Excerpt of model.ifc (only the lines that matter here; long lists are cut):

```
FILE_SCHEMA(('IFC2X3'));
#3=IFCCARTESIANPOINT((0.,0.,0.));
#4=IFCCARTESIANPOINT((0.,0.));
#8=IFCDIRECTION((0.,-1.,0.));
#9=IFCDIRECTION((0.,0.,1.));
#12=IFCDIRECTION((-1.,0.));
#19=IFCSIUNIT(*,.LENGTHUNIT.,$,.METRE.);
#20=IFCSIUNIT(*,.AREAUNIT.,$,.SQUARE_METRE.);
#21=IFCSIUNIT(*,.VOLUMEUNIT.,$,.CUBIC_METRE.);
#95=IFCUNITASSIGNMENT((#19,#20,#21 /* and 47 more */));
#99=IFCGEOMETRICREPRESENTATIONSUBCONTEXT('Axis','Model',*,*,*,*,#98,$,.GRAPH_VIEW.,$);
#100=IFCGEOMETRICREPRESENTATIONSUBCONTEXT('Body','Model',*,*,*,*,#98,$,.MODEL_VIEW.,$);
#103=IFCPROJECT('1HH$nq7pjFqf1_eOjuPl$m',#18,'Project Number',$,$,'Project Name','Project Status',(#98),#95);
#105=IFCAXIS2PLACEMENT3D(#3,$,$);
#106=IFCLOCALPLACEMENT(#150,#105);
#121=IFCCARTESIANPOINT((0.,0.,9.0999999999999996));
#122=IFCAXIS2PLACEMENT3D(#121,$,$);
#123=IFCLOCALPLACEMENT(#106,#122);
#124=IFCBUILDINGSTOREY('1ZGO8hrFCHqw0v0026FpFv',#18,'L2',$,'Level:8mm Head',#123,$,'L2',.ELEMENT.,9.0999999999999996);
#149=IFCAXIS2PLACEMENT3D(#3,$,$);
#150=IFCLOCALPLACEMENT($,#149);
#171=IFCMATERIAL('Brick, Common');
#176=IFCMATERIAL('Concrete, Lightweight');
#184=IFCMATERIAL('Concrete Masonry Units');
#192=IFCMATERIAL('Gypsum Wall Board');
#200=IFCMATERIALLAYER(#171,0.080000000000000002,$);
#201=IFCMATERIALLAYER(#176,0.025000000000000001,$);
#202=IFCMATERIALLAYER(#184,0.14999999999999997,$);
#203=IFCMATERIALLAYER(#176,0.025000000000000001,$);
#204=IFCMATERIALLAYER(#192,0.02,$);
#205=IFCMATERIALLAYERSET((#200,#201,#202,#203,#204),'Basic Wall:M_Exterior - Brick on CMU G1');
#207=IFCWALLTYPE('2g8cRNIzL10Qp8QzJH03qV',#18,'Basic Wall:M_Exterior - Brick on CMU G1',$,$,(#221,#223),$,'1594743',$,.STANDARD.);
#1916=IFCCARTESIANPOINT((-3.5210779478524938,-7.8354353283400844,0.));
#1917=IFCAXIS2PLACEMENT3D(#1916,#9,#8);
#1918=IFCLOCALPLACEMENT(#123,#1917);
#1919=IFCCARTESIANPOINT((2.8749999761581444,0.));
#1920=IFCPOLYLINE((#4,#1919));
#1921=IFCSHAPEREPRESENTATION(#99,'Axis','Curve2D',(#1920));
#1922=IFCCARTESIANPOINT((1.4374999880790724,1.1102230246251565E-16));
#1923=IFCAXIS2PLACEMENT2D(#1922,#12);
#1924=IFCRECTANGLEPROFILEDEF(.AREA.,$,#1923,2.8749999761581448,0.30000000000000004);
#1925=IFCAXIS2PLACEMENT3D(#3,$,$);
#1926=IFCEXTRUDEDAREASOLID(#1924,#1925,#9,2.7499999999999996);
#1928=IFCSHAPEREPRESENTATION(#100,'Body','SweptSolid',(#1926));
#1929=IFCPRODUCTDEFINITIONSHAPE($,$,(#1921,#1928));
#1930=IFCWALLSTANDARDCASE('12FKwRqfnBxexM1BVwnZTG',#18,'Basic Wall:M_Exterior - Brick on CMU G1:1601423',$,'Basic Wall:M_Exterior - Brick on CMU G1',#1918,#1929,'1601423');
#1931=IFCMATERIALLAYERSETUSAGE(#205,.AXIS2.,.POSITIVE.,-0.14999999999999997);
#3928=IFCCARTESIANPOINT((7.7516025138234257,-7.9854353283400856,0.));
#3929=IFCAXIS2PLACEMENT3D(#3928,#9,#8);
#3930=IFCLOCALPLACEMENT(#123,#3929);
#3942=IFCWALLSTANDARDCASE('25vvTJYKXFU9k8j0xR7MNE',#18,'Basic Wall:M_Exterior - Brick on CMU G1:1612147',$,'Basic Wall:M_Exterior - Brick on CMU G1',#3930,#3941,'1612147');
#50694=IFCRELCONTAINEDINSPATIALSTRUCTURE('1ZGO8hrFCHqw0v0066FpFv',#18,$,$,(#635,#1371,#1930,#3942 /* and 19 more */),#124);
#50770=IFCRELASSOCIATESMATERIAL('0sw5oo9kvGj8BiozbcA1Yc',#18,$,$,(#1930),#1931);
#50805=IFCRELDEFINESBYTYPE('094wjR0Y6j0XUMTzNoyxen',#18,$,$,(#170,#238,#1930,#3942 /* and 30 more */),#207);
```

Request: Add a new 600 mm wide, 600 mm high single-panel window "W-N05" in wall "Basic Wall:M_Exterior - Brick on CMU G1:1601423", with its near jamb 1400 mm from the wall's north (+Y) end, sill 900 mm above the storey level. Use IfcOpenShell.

```python
import numpy as np
import ifcopenshell
import ifcopenshell.api.feature
import ifcopenshell.api.geometry
import ifcopenshell.api.root
import ifcopenshell.api.spatial
import ifcopenshell.api.type
import ifcopenshell.geom
import ifcopenshell.util.element
import ifcopenshell.util.placement
import ifcopenshell.util.representation
import ifcopenshell.util.shape
import ifcopenshell.util.unit

model = ifcopenshell.open("model.ifc")
unit_scale = ifcopenshell.util.unit.calculate_unit_scale(model)
settings = ifcopenshell.geom.settings()


def volume(element):
    """Net volume in cubic metres, openings subtracted."""
    shape = ifcopenshell.geom.create_shape(settings, element)
    return ifcopenshell.util.shape.get_volume(shape.geometry)


wall = model.by_guid("12FKwRqfnBxexM1BVwnZTG")
storey = ifcopenshell.util.element.get_container(wall, ifc_class="IfcBuildingStorey")
context = ifcopenshell.util.representation.get_context(model, "Model", "Body", "MODEL_VIEW")
before = volume(wall)

width, height, from_end, sill = 0.6, 0.6, 1.4, 0.9  # metres

# The wall runs along its own X axis, and the end named is its -X end.
wall_shape = ifcopenshell.geom.create_shape(settings, wall)
x, y, z = ifcopenshell.util.shape.get_vertices(wall_shape.geometry).T
start = x.min() + from_end
face, thickness = float(y.min()), float(y.max() - y.min())
wall_matrix = ifcopenshell.util.placement.get_local_placement(wall.ObjectPlacement)
level = ifcopenshell.util.placement.get_local_placement(storey.ObjectPlacement)[2, 3]


def in_wall(x, y):
    """Placement at x, y metres in the wall's axes, at sill height."""
    matrix = wall_matrix.copy()
    matrix[:, 3] = wall_matrix @ np.array([x / unit_scale, y / unit_scale, 0.0, 1.0])
    matrix[2, 3] = level + sill / unit_scale
    return matrix


# Opening: a box that overshoots both wall faces by 50 mm.
opening = ifcopenshell.api.root.create_entity(model, ifc_class="IfcOpeningElement")
box = ifcopenshell.api.geometry.add_wall_representation(
    model, context=context, length=width, height=height, thickness=thickness + 0.1
)
ifcopenshell.api.geometry.assign_representation(model, product=opening, representation=box)
ifcopenshell.api.geometry.edit_object_placement(model, product=opening, matrix=in_wall(start, face - 0.05), is_si=False)
ifcopenshell.api.feature.add_feature(model, feature=opening, element=wall)

window = ifcopenshell.api.root.create_entity(model, ifc_class="IfcWindow", name="W-N05")
window.OverallWidth, window.OverallHeight = width / unit_scale, height / unit_scale
body = ifcopenshell.api.geometry.add_window_representation(
    model,
    context=context,
    overall_width=window.OverallWidth,
    overall_height=window.OverallHeight,
    partition_type="SINGLE_PANEL",
)
ifcopenshell.api.geometry.assign_representation(model, product=window, representation=body)
ifcopenshell.api.spatial.assign_container(model, products=[window], relating_structure=storey)
fills = ifcopenshell.api.feature.add_filling(model, opening=opening, element=window)
fills.OwnerHistory = window.OwnerHistory  # required in IFC2X3

# IFC2X3 keeps the operation on the window style.
style = ifcopenshell.api.root.create_entity(model, ifc_class="IfcWindowStyle", name="W-N05")
style.OperationType, style.ConstructionType = "SINGLE_PANEL", "NOTDEFINED"
style.ParameterTakesPrecedence = style.Sizeable = False
ifcopenshell.api.type.assign_type(model, related_objects=[window], relating_type=style)

# Centre the window in the wall's thickness.
ifcopenshell.api.geometry.edit_object_placement(model, product=window, matrix=in_wall(start, face), is_si=False)
window_shape = ifcopenshell.geom.create_shape(settings, window)
depth = ifcopenshell.util.shape.get_vertices(window_shape.geometry)[:, 1]
offset = face + thickness / 2 - (depth.min() + depth.max()) / 2
ifcopenshell.api.geometry.edit_object_placement(model, product=window, matrix=in_wall(start, offset), is_si=False)

after = volume(wall)

print(f"wall volume {before:.3f} -> {after:.3f} m3")

model.write("model_v2.ifc")
```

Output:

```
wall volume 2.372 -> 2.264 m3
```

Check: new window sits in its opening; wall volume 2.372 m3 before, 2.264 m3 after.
